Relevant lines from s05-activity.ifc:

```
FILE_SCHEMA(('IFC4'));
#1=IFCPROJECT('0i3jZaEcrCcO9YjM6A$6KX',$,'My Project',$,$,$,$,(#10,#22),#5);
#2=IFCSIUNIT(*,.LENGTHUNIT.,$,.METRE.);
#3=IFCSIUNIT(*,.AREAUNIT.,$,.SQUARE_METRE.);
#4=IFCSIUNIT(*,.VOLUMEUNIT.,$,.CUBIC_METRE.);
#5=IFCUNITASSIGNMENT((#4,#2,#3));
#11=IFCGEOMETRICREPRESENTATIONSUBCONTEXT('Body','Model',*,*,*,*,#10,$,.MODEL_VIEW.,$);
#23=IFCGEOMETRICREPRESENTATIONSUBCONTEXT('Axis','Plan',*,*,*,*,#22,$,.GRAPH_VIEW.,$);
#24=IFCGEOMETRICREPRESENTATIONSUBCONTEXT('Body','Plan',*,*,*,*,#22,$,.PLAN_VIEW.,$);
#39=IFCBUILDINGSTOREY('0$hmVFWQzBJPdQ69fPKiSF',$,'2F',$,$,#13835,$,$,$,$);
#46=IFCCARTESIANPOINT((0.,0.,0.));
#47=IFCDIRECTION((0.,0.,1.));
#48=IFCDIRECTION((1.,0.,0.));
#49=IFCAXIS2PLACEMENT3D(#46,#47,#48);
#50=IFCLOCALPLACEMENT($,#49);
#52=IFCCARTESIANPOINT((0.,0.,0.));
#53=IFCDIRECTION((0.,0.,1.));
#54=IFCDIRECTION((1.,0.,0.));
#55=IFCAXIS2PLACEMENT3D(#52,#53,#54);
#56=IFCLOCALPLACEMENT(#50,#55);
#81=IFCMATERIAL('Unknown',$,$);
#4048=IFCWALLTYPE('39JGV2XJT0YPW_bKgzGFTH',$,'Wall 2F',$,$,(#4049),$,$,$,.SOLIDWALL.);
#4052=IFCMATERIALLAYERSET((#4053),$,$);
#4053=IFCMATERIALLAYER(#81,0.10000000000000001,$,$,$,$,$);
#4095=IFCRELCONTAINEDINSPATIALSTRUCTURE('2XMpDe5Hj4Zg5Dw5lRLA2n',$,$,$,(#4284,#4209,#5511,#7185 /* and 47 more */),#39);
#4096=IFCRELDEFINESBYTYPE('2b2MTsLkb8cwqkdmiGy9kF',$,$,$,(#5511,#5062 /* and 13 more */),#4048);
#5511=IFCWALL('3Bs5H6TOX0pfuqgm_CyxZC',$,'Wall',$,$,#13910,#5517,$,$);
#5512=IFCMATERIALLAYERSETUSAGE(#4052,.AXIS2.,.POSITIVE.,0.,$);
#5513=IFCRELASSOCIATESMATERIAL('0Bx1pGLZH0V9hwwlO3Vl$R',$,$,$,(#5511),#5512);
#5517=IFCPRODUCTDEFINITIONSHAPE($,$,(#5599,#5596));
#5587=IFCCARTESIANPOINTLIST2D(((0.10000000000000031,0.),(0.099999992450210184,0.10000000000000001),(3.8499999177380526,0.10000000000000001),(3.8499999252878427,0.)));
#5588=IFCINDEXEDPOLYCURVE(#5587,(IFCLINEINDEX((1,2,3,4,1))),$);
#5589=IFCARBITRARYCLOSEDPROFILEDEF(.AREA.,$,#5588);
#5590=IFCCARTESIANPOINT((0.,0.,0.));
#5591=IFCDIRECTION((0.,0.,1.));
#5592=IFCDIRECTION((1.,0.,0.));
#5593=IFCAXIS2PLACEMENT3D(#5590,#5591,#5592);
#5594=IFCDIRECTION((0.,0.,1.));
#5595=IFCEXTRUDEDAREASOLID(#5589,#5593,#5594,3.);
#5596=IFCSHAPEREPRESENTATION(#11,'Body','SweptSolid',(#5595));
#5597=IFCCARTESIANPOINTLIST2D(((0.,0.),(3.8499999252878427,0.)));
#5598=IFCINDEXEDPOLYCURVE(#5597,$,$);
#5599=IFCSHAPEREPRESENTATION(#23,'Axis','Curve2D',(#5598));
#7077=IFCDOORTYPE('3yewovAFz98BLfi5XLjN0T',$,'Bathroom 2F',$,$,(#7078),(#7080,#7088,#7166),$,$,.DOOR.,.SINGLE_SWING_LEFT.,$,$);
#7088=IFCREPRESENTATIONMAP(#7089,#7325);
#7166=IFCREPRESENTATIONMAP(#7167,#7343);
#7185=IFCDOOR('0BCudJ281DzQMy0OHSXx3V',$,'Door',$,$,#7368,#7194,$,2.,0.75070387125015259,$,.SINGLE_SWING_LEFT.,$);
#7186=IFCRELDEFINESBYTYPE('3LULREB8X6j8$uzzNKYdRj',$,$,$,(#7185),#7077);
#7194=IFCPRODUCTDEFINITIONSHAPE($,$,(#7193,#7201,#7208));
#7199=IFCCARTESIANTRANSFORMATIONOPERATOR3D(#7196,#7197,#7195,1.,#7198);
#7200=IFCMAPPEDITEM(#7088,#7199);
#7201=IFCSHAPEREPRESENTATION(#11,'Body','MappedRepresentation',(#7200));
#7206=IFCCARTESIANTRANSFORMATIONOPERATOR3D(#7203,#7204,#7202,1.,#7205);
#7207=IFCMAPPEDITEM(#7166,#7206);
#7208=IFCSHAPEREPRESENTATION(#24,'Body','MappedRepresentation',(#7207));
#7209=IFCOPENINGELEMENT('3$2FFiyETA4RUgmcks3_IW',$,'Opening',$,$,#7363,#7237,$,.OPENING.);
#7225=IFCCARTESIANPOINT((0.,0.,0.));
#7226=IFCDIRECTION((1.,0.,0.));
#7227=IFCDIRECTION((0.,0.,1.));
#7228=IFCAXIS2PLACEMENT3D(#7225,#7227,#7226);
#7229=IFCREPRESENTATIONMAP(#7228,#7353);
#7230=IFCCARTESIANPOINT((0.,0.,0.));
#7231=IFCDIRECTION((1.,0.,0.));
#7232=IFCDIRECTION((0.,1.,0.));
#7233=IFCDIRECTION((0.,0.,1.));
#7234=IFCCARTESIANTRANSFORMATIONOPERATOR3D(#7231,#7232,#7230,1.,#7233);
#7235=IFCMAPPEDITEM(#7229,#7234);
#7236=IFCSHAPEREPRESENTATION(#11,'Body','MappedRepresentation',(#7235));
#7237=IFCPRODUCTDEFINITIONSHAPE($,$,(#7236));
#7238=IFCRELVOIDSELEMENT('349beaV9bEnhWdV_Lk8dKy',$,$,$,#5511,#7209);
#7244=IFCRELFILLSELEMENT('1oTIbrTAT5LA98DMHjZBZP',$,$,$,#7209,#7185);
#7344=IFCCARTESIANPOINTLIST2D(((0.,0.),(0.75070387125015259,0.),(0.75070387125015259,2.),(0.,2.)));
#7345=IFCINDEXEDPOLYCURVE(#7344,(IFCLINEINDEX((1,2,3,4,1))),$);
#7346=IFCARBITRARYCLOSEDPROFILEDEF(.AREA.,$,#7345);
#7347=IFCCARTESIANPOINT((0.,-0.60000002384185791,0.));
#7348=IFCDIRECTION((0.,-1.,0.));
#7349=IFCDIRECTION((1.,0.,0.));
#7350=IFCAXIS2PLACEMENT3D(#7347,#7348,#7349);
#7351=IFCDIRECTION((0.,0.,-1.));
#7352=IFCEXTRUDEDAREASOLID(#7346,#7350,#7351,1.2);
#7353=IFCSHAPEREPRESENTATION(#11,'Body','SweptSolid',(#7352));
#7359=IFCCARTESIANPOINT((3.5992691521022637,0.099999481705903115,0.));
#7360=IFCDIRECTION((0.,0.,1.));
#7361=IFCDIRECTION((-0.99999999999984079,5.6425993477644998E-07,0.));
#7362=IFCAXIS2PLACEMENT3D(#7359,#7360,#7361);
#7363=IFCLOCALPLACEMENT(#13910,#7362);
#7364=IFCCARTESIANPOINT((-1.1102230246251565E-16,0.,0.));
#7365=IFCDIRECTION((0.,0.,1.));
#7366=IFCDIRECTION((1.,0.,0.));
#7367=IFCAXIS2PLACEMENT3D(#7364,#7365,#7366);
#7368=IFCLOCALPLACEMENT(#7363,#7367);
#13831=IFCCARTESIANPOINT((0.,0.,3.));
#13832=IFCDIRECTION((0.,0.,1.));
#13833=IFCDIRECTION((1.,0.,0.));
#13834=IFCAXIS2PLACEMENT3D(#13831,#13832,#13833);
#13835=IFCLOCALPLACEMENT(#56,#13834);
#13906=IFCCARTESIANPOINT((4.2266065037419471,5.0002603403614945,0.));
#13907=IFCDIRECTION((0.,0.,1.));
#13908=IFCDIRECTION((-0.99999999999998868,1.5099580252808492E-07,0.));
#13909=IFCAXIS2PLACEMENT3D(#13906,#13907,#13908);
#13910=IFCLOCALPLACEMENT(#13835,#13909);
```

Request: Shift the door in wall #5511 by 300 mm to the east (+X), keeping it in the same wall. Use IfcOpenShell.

```python
import ifcopenshell
import ifcopenshell.api.geometry
import ifcopenshell.util.placement

model = ifcopenshell.open("s05-activity.ifc")

door = model.by_guid("0BCudJ281DzQMy0OHSXx3V")
opening = door.FillsVoids[0].RelatingOpeningElement
wall = opening.VoidsElements[0].RelatingBuildingElement

wall_matrix = ifcopenshell.util.placement.get_local_placement(wall.ObjectPlacement)
shift = wall_matrix[:3, 0] * -0.3
before = ifcopenshell.util.placement.get_local_placement(door.ObjectPlacement)[:3, 3].copy()

# The door is placed relative to its opening, so it follows when the opening moves.
matrix = ifcopenshell.util.placement.get_local_placement(opening.ObjectPlacement)
matrix[:3, 3] += shift
ifcopenshell.api.geometry.edit_object_placement(
    model, product=opening, matrix=matrix, is_si=False, should_transform_children=True
)

after = ifcopenshell.util.placement.get_local_placement(door.ObjectPlacement)[:3, 3]
print("door moved by", (after - before).round(3) + 0.0)

model.write("s05-activity-out.ifc")
```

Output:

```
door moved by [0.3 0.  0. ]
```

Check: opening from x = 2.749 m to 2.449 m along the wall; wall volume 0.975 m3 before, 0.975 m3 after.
